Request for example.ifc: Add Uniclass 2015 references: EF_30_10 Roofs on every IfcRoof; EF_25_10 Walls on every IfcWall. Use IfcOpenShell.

First a look at what the model holds.

```python
import ifcopenshell

model = ifcopenshell.open("example.ifc")
print(model.schema)
print("classifications:", [c.Name for c in model.by_type("IfcClassification")])
for ifc_class in ("IfcDoor", "IfcRoof", "IfcStair", "IfcWall", "IfcWindow"):
    print(ifc_class, len(model.by_type(ifc_class)))
```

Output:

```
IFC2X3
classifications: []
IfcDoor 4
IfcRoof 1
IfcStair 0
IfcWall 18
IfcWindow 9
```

```python
import ifcopenshell
import ifcopenshell.api.classification

model = ifcopenshell.open("example.ifc")

# IFC2X3 requires Source and Edition and has no link from the project to the system.
system = model.create_entity("IfcClassification", Source="NBS", Edition="2015", Name="Uniclass 2015")

codes = {
    "IfcRoof": ("EF_30_10", "Roofs"),
    "IfcWall": ("EF_25_10", "Walls"),
}
for ifc_class, (code, name) in codes.items():
    products = model.by_type(ifc_class)
    ifcopenshell.api.classification.add_reference(
        model, products=products, classification=system, identification=code, name=name
    )
    print(code, len(products))

model.write("example-out.ifc")
```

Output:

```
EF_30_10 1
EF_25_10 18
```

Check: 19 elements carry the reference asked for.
